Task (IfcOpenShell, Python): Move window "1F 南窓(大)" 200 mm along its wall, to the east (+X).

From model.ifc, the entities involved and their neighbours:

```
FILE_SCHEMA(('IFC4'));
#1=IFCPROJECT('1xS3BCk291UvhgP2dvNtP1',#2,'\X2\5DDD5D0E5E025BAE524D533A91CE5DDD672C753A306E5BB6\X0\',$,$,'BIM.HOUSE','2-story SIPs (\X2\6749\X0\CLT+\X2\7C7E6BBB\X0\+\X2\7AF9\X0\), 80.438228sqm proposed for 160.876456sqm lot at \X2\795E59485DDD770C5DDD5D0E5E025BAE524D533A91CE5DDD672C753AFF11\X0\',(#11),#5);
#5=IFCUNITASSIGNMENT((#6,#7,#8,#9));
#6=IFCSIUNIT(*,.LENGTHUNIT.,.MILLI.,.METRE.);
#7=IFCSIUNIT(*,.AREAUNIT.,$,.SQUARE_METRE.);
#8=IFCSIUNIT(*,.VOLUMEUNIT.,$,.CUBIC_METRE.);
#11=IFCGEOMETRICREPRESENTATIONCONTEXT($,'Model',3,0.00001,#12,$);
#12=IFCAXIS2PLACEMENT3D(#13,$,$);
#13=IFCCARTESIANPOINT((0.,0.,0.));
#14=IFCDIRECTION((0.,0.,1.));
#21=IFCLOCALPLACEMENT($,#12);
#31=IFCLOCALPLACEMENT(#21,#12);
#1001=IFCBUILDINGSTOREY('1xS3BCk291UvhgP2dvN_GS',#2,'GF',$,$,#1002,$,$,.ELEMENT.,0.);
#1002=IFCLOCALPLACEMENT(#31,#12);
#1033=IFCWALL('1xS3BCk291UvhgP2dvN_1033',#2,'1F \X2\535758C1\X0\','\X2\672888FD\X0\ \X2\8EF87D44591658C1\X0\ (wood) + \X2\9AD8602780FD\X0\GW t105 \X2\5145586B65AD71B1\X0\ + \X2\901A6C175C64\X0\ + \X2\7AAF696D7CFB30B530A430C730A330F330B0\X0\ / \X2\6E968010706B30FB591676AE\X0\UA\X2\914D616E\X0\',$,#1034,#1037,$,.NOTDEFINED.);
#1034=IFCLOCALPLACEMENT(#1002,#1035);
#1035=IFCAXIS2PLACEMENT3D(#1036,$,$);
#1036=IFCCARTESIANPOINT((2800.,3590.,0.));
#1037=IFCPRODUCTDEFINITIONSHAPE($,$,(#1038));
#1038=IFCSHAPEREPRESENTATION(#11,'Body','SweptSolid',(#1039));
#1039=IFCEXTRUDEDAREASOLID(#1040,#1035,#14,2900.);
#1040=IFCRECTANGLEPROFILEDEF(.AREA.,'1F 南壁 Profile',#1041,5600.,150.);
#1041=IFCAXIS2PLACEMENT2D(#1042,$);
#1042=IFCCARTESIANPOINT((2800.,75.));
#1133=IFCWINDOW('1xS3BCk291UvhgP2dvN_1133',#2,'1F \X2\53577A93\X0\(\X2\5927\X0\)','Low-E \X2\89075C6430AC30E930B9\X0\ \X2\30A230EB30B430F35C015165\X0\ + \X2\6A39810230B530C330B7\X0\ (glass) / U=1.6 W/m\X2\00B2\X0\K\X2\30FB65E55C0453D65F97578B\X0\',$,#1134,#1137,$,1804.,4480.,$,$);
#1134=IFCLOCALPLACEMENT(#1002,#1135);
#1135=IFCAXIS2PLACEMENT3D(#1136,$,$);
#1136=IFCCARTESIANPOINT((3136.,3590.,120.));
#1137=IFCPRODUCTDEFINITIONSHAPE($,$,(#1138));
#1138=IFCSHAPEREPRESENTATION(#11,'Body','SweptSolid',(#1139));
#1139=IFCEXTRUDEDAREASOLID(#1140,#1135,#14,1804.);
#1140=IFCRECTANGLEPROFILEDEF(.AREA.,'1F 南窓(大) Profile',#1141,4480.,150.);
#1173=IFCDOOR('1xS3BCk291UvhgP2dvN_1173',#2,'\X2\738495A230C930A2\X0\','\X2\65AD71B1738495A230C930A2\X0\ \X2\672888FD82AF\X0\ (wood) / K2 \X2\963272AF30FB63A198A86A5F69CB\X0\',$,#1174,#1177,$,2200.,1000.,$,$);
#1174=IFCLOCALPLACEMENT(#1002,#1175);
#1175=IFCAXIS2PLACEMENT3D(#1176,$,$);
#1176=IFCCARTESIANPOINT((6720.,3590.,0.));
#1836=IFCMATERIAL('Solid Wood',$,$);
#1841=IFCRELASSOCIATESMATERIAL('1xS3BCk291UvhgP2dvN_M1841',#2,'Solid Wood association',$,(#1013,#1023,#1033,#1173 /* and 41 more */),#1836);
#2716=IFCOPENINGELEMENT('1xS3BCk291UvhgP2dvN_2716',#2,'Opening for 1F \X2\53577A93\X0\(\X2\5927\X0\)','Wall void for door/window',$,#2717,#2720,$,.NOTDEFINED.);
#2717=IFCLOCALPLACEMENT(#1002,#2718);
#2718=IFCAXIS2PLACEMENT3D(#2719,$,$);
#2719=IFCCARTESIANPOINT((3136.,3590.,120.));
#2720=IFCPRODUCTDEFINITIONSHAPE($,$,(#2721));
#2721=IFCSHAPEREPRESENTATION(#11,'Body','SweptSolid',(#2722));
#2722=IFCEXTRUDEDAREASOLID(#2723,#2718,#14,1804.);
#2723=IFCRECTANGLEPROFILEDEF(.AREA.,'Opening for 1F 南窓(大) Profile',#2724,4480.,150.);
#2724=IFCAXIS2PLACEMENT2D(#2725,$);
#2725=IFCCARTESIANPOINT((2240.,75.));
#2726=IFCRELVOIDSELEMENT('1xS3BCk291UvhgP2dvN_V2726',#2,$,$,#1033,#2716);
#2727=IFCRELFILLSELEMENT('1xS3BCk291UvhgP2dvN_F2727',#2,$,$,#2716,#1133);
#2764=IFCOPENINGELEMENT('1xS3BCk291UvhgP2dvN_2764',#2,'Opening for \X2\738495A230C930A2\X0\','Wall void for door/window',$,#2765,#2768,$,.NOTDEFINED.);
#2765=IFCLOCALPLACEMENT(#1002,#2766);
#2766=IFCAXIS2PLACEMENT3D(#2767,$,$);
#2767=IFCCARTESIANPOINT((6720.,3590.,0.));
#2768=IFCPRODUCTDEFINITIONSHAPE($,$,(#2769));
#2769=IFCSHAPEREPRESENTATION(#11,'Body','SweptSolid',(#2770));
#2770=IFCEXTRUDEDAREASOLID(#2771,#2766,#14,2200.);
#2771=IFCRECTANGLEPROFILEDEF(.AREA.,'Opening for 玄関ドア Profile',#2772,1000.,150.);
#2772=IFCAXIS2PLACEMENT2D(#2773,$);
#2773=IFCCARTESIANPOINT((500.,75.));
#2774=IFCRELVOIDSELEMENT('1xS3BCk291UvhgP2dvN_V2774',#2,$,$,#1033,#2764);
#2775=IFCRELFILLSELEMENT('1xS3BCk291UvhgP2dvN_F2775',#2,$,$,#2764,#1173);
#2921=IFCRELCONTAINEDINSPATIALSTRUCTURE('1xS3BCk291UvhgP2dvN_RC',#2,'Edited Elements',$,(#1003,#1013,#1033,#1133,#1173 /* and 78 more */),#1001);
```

```python
import ifcopenshell
import ifcopenshell.api.geometry
import ifcopenshell.util.placement
import ifcopenshell.util.unit

model = ifcopenshell.open("model.ifc")
unit_scale = ifcopenshell.util.unit.calculate_unit_scale(model)

window = model.by_id(1133)
opening = window.FillsVoids[0].RelatingOpeningElement
wall = opening.VoidsElements[0].RelatingBuildingElement

wall_matrix = ifcopenshell.util.placement.get_local_placement(wall.ObjectPlacement)
shift = wall_matrix[:3, 0] * 0.2 / unit_scale
before = ifcopenshell.util.placement.get_local_placement(window.ObjectPlacement)[:3, 3].copy()

# The window is not placed relative to its opening, so move both.
for product in (opening, window):
    matrix = ifcopenshell.util.placement.get_local_placement(product.ObjectPlacement)
    matrix[:3, 3] += shift
    ifcopenshell.api.geometry.edit_object_placement(model, product=product, matrix=matrix, is_si=False)

after = ifcopenshell.util.placement.get_local_placement(window.ObjectPlacement)[:3, 3]
print("window moved by", (after - before).round(3) + 0.0)

model.write("model_edited.ifc")
```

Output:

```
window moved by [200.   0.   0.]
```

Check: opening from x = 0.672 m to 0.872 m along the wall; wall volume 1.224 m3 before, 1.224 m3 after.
